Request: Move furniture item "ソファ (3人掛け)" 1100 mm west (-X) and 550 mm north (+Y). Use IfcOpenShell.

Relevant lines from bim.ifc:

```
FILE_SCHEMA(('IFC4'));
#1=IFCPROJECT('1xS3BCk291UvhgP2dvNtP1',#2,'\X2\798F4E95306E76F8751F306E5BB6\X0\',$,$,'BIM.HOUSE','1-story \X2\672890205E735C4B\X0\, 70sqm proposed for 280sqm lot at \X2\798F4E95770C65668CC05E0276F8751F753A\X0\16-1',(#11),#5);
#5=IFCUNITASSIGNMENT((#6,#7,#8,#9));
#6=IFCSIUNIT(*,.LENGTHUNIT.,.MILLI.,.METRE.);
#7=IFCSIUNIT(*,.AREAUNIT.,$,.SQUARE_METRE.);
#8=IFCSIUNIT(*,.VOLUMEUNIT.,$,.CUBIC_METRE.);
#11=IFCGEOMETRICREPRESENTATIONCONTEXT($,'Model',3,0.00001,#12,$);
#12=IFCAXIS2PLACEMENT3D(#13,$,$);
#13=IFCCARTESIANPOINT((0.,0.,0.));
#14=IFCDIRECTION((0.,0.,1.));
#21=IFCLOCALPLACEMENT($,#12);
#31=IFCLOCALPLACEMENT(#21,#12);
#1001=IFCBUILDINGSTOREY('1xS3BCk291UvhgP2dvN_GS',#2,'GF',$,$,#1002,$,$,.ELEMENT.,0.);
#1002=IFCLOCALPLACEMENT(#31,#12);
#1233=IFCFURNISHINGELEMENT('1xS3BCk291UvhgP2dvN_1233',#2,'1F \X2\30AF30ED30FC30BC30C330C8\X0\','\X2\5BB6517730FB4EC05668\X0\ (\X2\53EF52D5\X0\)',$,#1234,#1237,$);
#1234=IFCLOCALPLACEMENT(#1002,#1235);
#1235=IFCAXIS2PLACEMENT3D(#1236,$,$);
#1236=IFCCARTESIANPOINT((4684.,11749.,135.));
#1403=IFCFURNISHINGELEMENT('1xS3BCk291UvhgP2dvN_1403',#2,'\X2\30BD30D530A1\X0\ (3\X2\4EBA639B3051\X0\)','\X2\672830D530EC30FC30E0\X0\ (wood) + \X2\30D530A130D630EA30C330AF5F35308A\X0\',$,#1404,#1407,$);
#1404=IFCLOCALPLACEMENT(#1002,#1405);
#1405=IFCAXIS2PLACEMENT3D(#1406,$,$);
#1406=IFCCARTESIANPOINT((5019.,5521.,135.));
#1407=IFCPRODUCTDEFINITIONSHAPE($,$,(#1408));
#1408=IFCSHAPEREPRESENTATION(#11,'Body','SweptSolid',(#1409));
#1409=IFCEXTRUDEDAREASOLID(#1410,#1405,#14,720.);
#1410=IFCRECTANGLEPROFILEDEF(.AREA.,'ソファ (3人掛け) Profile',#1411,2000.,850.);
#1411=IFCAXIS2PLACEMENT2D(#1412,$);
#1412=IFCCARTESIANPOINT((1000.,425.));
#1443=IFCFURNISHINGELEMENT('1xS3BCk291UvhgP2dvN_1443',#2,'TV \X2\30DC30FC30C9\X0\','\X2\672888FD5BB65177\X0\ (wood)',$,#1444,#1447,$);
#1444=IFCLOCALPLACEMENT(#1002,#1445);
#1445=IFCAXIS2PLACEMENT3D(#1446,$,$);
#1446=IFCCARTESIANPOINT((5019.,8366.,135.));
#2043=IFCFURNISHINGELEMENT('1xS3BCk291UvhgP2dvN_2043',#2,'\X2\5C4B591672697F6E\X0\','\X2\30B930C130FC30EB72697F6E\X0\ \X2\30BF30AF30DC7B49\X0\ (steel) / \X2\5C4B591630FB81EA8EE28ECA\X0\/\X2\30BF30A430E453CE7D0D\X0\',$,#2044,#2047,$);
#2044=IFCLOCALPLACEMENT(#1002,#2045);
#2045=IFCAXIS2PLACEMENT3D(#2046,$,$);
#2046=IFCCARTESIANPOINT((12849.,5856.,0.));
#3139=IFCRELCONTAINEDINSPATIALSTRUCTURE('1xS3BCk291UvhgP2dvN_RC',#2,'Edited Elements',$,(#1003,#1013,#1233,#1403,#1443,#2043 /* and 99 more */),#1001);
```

```python
import ifcopenshell
import ifcopenshell.api.geometry
import ifcopenshell.util.placement
import ifcopenshell.util.unit

model = ifcopenshell.open("bim.ifc")
unit_scale = ifcopenshell.util.unit.calculate_unit_scale(model)

item = model.by_guid("1xS3BCk291UvhgP2dvN_1403")
matrix = ifcopenshell.util.placement.get_local_placement(item.ObjectPlacement)
matrix[0, 3] -= 1.1 / unit_scale
matrix[1, 3] += 0.55 / unit_scale
ifcopenshell.api.geometry.edit_object_placement(model, product=item, matrix=matrix, is_si=False)

print(ifcopenshell.util.placement.get_local_placement(item.ObjectPlacement).round(3) + 0.0)

model.write("bim-out.ifc")
```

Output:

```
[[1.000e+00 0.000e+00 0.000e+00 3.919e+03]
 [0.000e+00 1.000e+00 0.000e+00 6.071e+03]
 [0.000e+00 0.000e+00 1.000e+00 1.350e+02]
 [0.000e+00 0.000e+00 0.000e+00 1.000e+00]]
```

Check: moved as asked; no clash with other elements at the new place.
